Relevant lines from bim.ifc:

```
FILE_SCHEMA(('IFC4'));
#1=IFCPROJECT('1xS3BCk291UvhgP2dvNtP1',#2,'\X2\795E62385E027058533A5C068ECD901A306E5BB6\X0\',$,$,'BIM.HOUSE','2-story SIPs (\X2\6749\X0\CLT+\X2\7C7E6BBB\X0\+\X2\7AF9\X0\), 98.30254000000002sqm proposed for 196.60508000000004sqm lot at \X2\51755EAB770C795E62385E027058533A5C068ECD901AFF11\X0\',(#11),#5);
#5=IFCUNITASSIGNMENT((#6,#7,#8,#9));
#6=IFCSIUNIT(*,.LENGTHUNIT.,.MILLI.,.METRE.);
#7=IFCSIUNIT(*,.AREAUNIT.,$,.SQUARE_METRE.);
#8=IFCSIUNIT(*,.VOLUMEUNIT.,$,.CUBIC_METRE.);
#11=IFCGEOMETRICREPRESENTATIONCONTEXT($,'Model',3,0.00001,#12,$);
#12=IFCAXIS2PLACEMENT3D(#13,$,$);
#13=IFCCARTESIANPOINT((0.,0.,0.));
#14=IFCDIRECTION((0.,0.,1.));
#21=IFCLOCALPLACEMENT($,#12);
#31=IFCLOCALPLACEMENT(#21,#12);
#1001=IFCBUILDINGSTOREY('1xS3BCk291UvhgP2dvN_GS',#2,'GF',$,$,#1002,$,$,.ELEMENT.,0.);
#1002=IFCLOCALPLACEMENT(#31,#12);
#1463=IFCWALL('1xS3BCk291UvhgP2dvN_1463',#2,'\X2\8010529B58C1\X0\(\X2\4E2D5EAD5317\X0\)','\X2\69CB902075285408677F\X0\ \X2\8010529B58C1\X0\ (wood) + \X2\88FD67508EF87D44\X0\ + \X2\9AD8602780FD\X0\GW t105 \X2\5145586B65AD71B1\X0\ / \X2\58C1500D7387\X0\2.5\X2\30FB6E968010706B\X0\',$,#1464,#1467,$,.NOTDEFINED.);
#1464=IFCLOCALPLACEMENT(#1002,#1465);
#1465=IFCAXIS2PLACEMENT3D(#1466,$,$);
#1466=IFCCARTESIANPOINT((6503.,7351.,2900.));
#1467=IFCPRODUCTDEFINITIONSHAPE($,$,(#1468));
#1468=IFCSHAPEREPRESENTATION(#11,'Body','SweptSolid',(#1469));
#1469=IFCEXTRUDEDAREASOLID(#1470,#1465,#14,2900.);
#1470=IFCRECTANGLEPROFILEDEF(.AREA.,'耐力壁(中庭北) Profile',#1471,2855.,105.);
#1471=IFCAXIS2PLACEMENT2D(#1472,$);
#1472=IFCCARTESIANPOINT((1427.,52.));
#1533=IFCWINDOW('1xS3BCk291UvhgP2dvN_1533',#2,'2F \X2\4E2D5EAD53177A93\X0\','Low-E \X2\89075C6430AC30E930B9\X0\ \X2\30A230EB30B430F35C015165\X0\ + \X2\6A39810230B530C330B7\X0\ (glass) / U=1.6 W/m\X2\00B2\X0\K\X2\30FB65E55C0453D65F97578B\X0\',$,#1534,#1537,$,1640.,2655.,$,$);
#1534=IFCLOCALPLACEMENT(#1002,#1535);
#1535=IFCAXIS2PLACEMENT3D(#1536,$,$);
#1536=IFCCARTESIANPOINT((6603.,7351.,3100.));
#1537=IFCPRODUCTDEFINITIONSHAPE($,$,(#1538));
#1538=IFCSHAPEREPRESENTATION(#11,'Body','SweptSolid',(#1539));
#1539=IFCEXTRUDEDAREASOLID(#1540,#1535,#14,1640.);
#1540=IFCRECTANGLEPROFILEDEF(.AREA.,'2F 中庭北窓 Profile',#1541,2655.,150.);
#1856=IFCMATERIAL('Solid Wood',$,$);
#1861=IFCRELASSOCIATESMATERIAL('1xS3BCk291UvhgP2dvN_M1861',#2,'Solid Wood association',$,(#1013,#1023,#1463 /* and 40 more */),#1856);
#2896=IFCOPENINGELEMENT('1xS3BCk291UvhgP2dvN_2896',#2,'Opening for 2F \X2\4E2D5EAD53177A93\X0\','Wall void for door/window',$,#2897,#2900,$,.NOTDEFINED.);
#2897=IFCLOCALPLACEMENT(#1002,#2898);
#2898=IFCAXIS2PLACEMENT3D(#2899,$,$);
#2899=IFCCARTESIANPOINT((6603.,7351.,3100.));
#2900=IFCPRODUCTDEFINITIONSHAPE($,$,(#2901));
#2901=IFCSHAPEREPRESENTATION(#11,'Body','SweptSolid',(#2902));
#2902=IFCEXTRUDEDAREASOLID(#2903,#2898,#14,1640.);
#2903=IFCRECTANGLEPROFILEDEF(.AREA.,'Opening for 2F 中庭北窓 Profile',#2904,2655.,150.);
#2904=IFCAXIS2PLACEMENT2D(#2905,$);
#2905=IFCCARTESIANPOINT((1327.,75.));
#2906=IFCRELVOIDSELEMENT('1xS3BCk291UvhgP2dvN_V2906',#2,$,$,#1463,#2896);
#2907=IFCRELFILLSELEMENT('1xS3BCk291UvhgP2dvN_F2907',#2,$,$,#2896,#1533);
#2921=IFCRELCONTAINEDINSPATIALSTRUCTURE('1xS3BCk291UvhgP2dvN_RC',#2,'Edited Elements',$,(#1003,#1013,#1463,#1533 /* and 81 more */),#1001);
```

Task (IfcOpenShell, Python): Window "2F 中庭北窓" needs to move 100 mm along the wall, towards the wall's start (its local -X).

```python
import ifcopenshell
import ifcopenshell.api.geometry
import ifcopenshell.util.placement
import ifcopenshell.util.unit

model = ifcopenshell.open("bim.ifc")
unit_scale = ifcopenshell.util.unit.calculate_unit_scale(model)

window = model.by_guid("1xS3BCk291UvhgP2dvN_1533")
opening = window.FillsVoids[0].RelatingOpeningElement
wall = opening.VoidsElements[0].RelatingBuildingElement

wall_matrix = ifcopenshell.util.placement.get_local_placement(wall.ObjectPlacement)
shift = wall_matrix[:3, 0] * -0.1 / unit_scale
before = ifcopenshell.util.placement.get_local_placement(window.ObjectPlacement)[:3, 3].copy()

# The window is not placed relative to its opening, so move both.
for product in (opening, window):
    matrix = ifcopenshell.util.placement.get_local_placement(product.ObjectPlacement)
    matrix[:3, 3] += shift
    ifcopenshell.api.geometry.edit_object_placement(model, product=product, matrix=matrix, is_si=False)

after = ifcopenshell.util.placement.get_local_placement(window.ObjectPlacement)[:3, 3]
print("window moved by", (after - before).round(3) + 0.0)

model.write("bim_rev.ifc")
```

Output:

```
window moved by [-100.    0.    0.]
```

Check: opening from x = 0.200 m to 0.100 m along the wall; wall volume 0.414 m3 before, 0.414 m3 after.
